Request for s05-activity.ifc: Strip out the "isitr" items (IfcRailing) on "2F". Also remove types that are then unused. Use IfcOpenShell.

First a look at what the model holds.

```python
import ifcopenshell
import ifcopenshell.util.element

model = ifcopenshell.open("s05-activity.ifc")
print(model.schema)
storey = next(s for s in model.by_type("IfcBuildingStorey") if s.Name == "2F")
railings = [e for e in ifcopenshell.util.element.get_decomposition(storey) if e.is_a("IfcRailing")]
seen = {}
for e in railings:
    element_type = ifcopenshell.util.element.get_type(e)
    name = element_type.Name if element_type not in (None, e) else None
    seen[name] = seen.get(name, 0) + 1
for name, count in sorted(seen.items(), key=str):
    print(count, "x", name)
```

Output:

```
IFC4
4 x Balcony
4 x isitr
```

```python
import ifcopenshell
import ifcopenshell.api.root
import ifcopenshell.util.element

model = ifcopenshell.open("s05-activity.ifc")

storey = next(s for s in model.by_type("IfcBuildingStorey") if s.Name == "2F")
railings = [e for e in ifcopenshell.util.element.get_decomposition(storey) if e.is_a("IfcRailing")]
targets = [e for e in railings if (t := ifcopenshell.util.element.get_type(e)) not in (None, e) and t.Name == "isitr"]
types = {ifcopenshell.util.element.get_type(e) for e in targets} - {None, *targets}

for e in targets:
    ifcopenshell.api.root.remove_product(model, product=e)
print(len(targets), "removed")

unused = [t for t in types if not ifcopenshell.util.element.get_types(t)]
for t in unused:
    ifcopenshell.api.root.remove_product(model, product=t)
print(len(unused), "unused types removed")

model.write("s05-activity_rev.ifc")
```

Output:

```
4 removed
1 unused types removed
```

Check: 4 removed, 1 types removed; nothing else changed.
